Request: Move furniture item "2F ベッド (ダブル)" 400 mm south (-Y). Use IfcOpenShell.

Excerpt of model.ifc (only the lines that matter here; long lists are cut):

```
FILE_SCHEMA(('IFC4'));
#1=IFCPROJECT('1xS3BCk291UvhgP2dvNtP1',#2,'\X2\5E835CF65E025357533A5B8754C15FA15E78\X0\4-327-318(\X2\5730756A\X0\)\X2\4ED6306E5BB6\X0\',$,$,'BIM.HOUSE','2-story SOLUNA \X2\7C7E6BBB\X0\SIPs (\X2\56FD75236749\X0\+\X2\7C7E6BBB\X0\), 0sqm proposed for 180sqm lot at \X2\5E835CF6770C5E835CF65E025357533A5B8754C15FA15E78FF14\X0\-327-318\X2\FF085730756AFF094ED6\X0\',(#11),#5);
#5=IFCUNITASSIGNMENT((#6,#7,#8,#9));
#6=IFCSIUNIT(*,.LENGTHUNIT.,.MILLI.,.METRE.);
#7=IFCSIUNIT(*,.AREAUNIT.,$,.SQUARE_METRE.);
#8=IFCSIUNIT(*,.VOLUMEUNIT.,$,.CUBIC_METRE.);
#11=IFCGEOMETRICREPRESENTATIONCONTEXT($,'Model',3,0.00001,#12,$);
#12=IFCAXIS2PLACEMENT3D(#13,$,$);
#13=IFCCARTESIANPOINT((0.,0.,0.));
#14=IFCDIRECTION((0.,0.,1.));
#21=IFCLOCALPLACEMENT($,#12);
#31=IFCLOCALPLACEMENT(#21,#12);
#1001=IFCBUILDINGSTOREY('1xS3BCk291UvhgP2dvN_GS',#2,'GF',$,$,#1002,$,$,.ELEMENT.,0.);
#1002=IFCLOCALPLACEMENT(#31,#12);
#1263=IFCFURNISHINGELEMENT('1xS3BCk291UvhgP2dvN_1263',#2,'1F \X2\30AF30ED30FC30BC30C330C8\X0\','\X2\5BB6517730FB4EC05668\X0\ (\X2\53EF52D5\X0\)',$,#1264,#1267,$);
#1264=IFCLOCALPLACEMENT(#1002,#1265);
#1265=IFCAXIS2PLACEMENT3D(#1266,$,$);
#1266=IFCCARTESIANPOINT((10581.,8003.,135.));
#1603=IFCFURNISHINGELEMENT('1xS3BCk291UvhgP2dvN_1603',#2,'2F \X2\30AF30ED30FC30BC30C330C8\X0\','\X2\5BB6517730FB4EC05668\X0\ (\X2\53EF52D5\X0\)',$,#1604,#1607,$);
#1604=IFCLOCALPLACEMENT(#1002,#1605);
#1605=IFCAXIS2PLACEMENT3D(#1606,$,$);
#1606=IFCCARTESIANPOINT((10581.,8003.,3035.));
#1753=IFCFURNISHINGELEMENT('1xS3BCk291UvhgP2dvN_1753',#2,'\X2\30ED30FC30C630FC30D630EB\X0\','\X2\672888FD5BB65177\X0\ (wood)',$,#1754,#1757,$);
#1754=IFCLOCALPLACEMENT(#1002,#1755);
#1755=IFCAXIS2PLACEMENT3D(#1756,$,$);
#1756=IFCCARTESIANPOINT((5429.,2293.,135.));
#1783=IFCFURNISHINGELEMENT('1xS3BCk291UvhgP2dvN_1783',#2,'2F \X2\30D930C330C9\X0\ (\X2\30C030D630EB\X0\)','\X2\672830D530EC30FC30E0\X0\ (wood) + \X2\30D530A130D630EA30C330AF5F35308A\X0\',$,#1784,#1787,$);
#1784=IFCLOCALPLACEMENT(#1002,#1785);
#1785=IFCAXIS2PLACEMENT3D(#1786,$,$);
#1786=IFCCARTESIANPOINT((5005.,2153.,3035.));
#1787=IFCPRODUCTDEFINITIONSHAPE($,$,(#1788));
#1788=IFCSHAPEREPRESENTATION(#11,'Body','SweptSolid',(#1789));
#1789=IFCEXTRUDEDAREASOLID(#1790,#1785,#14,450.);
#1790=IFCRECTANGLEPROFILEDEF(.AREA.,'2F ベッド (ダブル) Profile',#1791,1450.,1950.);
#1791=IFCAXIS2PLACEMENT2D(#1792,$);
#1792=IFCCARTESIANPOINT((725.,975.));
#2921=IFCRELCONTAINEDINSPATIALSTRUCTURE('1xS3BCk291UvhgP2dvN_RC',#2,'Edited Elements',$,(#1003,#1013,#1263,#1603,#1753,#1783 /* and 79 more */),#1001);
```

```python
import ifcopenshell
import ifcopenshell.api.geometry
import ifcopenshell.util.placement
import ifcopenshell.util.unit

model = ifcopenshell.open("model.ifc")
unit_scale = ifcopenshell.util.unit.calculate_unit_scale(model)

item = model.by_id(1783)
matrix = ifcopenshell.util.placement.get_local_placement(item.ObjectPlacement)
matrix[1, 3] -= 0.4 / unit_scale
ifcopenshell.api.geometry.edit_object_placement(model, product=item, matrix=matrix, is_si=False)

print(ifcopenshell.util.placement.get_local_placement(item.ObjectPlacement).round(3) + 0.0)

model.write("model_updated.ifc")
```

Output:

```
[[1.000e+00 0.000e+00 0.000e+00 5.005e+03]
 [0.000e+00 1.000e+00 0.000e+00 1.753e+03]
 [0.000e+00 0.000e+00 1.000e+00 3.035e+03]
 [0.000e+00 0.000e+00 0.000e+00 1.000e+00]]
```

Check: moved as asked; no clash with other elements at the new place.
